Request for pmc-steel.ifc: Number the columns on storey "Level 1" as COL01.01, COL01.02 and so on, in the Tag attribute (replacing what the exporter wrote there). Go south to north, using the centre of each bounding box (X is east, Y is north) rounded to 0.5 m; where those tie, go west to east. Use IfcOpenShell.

First a look at what the model holds.

```python
import ifcopenshell
import ifcopenshell.util.element
import ifcopenshell.util.placement

model = ifcopenshell.open("pmc-steel.ifc")
print(model.schema)
storey = next(s for s in model.by_type("IfcBuildingStorey") if s.Name == "Level 1")
columns = [e for e in ifcopenshell.util.element.get_decomposition(storey) if e.is_a("IfcColumn")]
for e in sorted(columns, key=lambda e: e.id()):
    origin = ifcopenshell.util.placement.get_local_placement(e.ObjectPlacement)[:3, 3]
    print(e.id(), e.Tag, e.Name, origin.round(2) + 0.0, sep=" | ")
```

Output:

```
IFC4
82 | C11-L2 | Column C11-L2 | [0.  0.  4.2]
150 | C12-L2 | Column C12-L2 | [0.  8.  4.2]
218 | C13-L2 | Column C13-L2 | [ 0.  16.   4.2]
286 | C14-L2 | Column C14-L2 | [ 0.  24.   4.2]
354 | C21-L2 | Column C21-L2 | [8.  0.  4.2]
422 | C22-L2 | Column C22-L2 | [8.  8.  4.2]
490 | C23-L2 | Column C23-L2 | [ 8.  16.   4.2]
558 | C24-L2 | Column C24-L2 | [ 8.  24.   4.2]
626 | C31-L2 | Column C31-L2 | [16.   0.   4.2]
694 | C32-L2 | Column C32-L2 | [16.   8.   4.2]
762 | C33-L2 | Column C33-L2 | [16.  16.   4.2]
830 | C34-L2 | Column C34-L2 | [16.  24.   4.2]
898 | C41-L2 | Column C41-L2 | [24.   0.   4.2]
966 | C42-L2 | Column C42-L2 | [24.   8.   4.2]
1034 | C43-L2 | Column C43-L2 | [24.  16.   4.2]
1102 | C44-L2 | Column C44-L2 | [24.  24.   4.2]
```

```python
import ifcopenshell
import ifcopenshell.geom
import ifcopenshell.util.element
import ifcopenshell.util.shape

model = ifcopenshell.open("pmc-steel.ifc")
settings = ifcopenshell.geom.settings()
settings.set("use-world-coords", True)


def centre(element):
    shape = ifcopenshell.geom.create_shape(settings, element)
    return ifcopenshell.util.shape.get_bbox_centroid(shape.geometry)


storey = next(s for s in model.by_type("IfcBuildingStorey") if s.Name == "Level 1")
columns = [e for e in ifcopenshell.util.element.get_decomposition(storey) if e.is_a("IfcColumn")]

# Insertion points can sit at a corner or the storey origin, so sort by the geometry (in metres).
centres = {e: centre(e) for e in columns}
columns.sort(key=lambda e: (round(centres[e][1] / 0.5), centres[e][0]))

for i, e in enumerate(columns, start=1):
    number = f"COL01.{i:02d}"
    e.Tag = number
    print(e.id(), number)

model.write("pmc-steel_v2.ifc")
```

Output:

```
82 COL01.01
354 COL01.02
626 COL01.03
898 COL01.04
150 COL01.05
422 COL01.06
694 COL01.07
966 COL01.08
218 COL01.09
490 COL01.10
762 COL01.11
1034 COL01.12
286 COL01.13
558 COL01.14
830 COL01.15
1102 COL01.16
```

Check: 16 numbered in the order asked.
